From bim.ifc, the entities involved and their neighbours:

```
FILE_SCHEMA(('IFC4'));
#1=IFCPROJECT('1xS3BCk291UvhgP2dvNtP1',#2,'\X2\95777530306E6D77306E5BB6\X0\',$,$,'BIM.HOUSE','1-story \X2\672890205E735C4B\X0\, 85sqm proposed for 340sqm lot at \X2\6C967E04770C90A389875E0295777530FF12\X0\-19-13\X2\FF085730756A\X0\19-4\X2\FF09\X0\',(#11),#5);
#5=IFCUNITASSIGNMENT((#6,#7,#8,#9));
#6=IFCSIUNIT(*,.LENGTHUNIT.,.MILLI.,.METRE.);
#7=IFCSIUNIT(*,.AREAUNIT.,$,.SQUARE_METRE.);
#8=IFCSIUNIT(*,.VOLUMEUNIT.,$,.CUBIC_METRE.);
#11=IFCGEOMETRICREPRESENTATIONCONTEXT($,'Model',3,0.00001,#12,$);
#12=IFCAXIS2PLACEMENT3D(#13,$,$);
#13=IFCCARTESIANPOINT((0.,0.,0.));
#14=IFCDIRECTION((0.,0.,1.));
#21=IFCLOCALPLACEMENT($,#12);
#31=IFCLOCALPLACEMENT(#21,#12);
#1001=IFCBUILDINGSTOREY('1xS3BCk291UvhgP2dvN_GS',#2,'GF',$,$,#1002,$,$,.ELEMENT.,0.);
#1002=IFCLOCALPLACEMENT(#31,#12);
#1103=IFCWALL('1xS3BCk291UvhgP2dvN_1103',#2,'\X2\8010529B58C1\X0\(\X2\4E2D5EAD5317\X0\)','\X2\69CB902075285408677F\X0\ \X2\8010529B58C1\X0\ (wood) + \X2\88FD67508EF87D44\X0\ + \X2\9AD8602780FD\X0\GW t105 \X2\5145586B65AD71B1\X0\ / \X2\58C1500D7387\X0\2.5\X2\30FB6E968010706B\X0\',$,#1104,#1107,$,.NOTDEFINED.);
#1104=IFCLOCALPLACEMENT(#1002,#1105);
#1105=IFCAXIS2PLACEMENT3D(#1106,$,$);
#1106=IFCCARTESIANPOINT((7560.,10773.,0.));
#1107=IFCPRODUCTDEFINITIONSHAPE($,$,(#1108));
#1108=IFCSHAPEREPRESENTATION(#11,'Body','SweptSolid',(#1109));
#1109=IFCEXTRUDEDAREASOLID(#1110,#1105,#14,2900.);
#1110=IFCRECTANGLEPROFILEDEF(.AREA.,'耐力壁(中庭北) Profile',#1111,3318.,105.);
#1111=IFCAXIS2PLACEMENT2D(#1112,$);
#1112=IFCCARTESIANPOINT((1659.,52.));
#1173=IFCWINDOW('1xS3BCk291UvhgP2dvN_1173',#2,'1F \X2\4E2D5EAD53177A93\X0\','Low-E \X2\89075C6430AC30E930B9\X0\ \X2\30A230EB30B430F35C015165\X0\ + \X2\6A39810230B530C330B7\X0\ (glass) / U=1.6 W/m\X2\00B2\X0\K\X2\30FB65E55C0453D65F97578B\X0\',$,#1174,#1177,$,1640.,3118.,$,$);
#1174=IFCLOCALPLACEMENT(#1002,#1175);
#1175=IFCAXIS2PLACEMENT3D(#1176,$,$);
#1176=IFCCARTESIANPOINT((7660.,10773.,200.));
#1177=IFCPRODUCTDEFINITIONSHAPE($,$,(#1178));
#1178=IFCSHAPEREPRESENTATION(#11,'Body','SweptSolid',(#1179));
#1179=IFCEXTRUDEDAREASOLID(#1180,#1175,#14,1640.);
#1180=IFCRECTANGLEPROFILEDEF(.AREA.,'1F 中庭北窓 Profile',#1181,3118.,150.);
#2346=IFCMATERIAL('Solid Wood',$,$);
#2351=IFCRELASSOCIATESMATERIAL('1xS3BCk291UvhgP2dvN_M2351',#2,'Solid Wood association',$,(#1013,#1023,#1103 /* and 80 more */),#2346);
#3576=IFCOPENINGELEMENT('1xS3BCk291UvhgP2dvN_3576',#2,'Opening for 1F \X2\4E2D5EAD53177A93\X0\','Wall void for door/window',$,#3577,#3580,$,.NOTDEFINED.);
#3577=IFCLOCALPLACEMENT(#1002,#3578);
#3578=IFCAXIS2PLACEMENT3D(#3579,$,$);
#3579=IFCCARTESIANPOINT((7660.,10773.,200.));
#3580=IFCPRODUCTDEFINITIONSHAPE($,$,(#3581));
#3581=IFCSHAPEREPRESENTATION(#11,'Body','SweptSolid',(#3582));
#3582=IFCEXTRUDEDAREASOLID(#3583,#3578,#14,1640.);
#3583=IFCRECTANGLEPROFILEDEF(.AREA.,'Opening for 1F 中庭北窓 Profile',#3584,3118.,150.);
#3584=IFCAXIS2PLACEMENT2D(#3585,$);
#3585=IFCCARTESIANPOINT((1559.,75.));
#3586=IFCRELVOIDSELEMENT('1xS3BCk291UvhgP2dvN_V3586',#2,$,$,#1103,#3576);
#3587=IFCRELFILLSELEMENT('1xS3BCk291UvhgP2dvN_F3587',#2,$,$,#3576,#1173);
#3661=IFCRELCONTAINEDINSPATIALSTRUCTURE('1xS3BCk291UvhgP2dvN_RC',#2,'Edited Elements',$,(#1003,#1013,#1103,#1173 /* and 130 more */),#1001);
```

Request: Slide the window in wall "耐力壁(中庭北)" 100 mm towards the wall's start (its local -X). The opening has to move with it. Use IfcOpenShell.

```python
import ifcopenshell
import ifcopenshell.api.geometry
import ifcopenshell.util.placement

model = ifcopenshell.open("bim.ifc")

window = model.by_guid("1xS3BCk291UvhgP2dvN_1173")
opening = window.FillsVoids[0].RelatingOpeningElement
wall = opening.VoidsElements[0].RelatingBuildingElement

wall_matrix = ifcopenshell.util.placement.get_local_placement(wall.ObjectPlacement)
shift = wall_matrix[:3, 0] * -100.0
before = ifcopenshell.util.placement.get_local_placement(window.ObjectPlacement)[:3, 3].copy()

# The window is not placed relative to its opening, so move both.
for product in (opening, window):
    matrix = ifcopenshell.util.placement.get_local_placement(product.ObjectPlacement)
    matrix[:3, 3] += shift
    ifcopenshell.api.geometry.edit_object_placement(model, product=product, matrix=matrix, is_si=False)

after = ifcopenshell.util.placement.get_local_placement(window.ObjectPlacement)[:3, 3]
print("window moved by", (after - before).round(3) + 0.0)

model.write("bim_updated.ifc")
```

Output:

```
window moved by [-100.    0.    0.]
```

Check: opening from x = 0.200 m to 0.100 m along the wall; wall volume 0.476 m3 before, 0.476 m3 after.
